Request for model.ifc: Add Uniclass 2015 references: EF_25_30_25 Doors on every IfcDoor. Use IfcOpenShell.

First a look at what the model holds.

```python
import ifcopenshell

model = ifcopenshell.open("model.ifc")
print(model.schema)
print("classifications:", [c.Name for c in model.by_type("IfcClassification")])
for ifc_class in ("IfcDoor", "IfcRoof", "IfcStair", "IfcWall", "IfcWindow"):
    print(ifc_class, len(model.by_type(ifc_class)))
```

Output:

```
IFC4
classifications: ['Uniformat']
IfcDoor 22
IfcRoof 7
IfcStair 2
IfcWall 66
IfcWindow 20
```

```python
import ifcopenshell
import ifcopenshell.api.classification

model = ifcopenshell.open("model.ifc")

system = ifcopenshell.api.classification.add_classification(model, classification="Uniclass 2015")

codes = {
    "IfcDoor": ("EF_25_30_25", "Doors"),
}
for ifc_class, (code, name) in codes.items():
    products = model.by_type(ifc_class)
    ifcopenshell.api.classification.add_reference(
        model, products=products, classification=system, identification=code, name=name
    )
    print(code, len(products))

model.write("model-out.ifc")
```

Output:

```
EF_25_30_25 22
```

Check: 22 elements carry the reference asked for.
